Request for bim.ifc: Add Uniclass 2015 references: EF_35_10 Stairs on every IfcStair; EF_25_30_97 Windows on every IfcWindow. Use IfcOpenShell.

First a look at what the model holds.

```python
import ifcopenshell

model = ifcopenshell.open("bim.ifc")
print(model.schema)
print("classifications:", [c.Name for c in model.by_type("IfcClassification")])
for ifc_class in ("IfcDoor", "IfcRoof", "IfcStair", "IfcWall", "IfcWindow"):
    print(ifc_class, len(model.by_type(ifc_class)))
```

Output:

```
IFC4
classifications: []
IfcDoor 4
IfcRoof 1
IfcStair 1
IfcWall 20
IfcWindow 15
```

```python
import ifcopenshell
import ifcopenshell.api.classification

model = ifcopenshell.open("bim.ifc")

system = ifcopenshell.api.classification.add_classification(model, classification="Uniclass 2015")

codes = {
    "IfcStair": ("EF_35_10", "Stairs"),
    "IfcWindow": ("EF_25_30_97", "Windows"),
}
for ifc_class, (code, name) in codes.items():
    products = model.by_type(ifc_class)
    ifcopenshell.api.classification.add_reference(
        model, products=products, classification=system, identification=code, name=name
    )
    print(code, len(products))

model.write("bim_edited.ifc")
```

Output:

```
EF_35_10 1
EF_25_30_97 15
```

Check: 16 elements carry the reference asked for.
